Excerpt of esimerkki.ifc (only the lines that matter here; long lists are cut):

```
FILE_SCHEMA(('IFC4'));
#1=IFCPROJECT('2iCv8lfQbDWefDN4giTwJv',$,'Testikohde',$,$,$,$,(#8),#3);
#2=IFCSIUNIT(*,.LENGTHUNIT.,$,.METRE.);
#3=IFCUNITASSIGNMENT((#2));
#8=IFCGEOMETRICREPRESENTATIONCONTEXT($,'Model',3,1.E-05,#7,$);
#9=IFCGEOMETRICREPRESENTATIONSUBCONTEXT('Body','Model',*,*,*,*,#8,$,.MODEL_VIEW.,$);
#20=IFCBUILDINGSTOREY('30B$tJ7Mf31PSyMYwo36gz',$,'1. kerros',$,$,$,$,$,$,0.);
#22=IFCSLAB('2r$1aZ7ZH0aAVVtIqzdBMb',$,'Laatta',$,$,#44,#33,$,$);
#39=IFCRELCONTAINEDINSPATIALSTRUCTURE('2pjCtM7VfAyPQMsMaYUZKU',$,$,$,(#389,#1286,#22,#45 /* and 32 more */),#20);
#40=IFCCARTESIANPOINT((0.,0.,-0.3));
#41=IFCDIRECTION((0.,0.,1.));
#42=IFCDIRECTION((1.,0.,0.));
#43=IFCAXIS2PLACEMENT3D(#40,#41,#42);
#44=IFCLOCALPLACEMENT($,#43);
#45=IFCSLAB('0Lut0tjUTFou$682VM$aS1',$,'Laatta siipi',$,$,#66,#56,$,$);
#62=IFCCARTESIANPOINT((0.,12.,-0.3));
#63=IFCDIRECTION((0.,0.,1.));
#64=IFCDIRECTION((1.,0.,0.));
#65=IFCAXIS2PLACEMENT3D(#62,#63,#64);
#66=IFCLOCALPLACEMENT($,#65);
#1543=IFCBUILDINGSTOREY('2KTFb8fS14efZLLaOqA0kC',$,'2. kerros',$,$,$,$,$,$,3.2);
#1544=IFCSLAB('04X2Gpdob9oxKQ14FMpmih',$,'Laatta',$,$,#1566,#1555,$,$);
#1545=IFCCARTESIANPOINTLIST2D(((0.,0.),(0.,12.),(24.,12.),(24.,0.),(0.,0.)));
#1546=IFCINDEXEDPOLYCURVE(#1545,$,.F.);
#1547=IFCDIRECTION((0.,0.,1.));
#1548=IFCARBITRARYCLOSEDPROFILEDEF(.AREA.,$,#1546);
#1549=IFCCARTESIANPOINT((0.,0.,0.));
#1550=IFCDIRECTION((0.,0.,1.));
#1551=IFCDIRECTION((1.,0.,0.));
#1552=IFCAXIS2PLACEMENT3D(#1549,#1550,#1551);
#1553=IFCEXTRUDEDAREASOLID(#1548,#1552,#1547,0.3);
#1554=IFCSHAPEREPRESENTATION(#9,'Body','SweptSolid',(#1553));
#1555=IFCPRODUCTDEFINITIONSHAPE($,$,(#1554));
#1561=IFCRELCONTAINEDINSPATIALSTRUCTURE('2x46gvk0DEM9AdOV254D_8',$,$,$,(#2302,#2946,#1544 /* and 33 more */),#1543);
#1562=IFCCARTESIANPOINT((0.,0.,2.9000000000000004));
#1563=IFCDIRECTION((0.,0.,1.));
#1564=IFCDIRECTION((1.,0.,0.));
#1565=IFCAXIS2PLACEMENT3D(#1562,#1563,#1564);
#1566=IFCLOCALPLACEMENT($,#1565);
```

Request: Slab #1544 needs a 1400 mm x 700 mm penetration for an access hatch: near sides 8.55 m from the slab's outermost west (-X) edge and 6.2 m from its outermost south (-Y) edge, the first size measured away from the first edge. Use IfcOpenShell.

```python
import numpy as np
import ifcopenshell
import ifcopenshell.api.feature
import ifcopenshell.api.geometry
import ifcopenshell.api.root
import ifcopenshell.geom
import ifcopenshell.util.placement
import ifcopenshell.util.representation
import ifcopenshell.util.shape
import ifcopenshell.util.unit

model = ifcopenshell.open("esimerkki.ifc")
unit_scale = ifcopenshell.util.unit.calculate_unit_scale(model)
settings = ifcopenshell.geom.settings()


def volume(element):
    """Net volume in cubic metres, openings subtracted."""
    shape = ifcopenshell.geom.create_shape(settings, element)
    return ifcopenshell.util.shape.get_volume(shape.geometry)


slab = model.by_id(1544)
before = volume(slab)

# Extent in the slab's own axes, in metres. The edges named are its -X and -Y sides.
slab_shape = ifcopenshell.geom.create_shape(settings, slab)
vertices = ifcopenshell.util.shape.get_vertices(slab_shape.geometry)
x_min, y_min, bottom = vertices.min(axis=0)
top = vertices[:, 2].max()

opening = ifcopenshell.api.root.create_entity(model, ifc_class="IfcOpeningElement", name="Access hatch opening", predefined_type="OPENING")
context = ifcopenshell.util.representation.get_context(model, "Model", "Body", "MODEL_VIEW")
width, depth = 1.4, 0.7
outline = [(0.0, 0.0), (width, 0.0), (width, depth), (0.0, depth), (0.0, 0.0)]
# Overshoot both faces by 50 mm so the cut is clean.
shape = ifcopenshell.api.geometry.add_slab_representation(
    model, context=context, depth=top - bottom + 0.1, polyline=outline
)
ifcopenshell.api.geometry.assign_representation(model, product=opening, representation=shape)

matrix = ifcopenshell.util.placement.get_local_placement(slab.ObjectPlacement)
matrix[:, 3] = matrix @ np.append(np.array([x_min + 8.55, y_min + 6.2, bottom - 0.05]) / unit_scale, 1.0)
ifcopenshell.api.geometry.edit_object_placement(model, product=opening, matrix=matrix, is_si=False)
ifcopenshell.api.feature.add_feature(model, feature=opening, element=slab)

after = volume(slab)

print(f"slab volume {before:.3f} -> {after:.3f} m3")

model.write("esimerkki_rev.ifc")
```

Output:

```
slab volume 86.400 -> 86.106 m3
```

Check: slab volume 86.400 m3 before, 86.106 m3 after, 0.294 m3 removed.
